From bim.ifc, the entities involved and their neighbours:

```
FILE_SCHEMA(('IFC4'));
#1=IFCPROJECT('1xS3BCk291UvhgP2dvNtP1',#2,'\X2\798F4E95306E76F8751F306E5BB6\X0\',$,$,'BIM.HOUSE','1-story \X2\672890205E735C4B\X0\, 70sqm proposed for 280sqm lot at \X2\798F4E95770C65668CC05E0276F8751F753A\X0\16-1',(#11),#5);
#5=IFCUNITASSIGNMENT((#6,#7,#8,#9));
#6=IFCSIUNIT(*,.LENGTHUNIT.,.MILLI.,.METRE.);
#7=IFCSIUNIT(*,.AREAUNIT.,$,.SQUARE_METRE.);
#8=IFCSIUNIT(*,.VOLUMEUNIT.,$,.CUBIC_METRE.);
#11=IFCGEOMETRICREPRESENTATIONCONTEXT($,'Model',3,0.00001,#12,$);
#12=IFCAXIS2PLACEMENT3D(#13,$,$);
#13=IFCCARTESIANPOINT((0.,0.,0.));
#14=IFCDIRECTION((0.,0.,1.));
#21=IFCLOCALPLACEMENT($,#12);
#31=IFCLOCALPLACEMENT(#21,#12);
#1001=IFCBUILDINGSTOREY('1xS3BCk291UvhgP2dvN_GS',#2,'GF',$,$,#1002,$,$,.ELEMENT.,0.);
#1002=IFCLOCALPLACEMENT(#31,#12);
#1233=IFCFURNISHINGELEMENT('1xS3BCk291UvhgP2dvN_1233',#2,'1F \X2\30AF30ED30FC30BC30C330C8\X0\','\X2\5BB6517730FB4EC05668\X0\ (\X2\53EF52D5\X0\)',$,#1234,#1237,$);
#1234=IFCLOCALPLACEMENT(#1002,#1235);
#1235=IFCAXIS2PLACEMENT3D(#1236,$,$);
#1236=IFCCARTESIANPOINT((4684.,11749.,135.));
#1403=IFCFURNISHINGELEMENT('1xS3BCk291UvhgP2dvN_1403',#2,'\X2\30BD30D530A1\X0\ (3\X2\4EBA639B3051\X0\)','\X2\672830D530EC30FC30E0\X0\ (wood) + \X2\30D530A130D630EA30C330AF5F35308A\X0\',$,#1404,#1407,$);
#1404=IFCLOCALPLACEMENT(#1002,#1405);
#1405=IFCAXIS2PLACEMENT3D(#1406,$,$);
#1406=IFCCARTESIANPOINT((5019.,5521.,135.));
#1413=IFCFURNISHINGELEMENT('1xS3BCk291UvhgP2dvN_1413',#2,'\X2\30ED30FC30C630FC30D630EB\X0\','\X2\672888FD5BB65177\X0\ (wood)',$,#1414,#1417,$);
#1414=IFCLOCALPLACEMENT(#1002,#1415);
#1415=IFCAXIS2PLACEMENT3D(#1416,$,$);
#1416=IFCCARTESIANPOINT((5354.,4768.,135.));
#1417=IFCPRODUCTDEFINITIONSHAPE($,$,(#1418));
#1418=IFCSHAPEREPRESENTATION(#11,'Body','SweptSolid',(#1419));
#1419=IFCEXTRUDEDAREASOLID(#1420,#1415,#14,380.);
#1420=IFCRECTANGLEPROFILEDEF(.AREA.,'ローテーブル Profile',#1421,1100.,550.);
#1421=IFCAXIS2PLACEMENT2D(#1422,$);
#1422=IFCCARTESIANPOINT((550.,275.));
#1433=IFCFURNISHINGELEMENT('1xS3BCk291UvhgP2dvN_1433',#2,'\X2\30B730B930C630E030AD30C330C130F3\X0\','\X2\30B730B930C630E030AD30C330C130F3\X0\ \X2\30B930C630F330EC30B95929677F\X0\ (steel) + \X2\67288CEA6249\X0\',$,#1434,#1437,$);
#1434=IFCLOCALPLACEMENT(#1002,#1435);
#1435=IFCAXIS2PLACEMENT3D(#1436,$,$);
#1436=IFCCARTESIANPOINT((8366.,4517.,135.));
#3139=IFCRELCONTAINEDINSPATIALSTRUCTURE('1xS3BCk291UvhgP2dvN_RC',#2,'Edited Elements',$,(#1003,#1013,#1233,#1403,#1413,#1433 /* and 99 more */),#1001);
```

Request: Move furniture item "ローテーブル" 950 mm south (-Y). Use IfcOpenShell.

```python
import ifcopenshell
import ifcopenshell.api.geometry
import ifcopenshell.util.placement
import ifcopenshell.util.unit

model = ifcopenshell.open("bim.ifc")
unit_scale = ifcopenshell.util.unit.calculate_unit_scale(model)

item = model.by_id(1413)
matrix = ifcopenshell.util.placement.get_local_placement(item.ObjectPlacement)
matrix[1, 3] -= 0.95 / unit_scale
ifcopenshell.api.geometry.edit_object_placement(model, product=item, matrix=matrix, is_si=False)

print(ifcopenshell.util.placement.get_local_placement(item.ObjectPlacement).round(3) + 0.0)

model.write("bim_updated.ifc")
```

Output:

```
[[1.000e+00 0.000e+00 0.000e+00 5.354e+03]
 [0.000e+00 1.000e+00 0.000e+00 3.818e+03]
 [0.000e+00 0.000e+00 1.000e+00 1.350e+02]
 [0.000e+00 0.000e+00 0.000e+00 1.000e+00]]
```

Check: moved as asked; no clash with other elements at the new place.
